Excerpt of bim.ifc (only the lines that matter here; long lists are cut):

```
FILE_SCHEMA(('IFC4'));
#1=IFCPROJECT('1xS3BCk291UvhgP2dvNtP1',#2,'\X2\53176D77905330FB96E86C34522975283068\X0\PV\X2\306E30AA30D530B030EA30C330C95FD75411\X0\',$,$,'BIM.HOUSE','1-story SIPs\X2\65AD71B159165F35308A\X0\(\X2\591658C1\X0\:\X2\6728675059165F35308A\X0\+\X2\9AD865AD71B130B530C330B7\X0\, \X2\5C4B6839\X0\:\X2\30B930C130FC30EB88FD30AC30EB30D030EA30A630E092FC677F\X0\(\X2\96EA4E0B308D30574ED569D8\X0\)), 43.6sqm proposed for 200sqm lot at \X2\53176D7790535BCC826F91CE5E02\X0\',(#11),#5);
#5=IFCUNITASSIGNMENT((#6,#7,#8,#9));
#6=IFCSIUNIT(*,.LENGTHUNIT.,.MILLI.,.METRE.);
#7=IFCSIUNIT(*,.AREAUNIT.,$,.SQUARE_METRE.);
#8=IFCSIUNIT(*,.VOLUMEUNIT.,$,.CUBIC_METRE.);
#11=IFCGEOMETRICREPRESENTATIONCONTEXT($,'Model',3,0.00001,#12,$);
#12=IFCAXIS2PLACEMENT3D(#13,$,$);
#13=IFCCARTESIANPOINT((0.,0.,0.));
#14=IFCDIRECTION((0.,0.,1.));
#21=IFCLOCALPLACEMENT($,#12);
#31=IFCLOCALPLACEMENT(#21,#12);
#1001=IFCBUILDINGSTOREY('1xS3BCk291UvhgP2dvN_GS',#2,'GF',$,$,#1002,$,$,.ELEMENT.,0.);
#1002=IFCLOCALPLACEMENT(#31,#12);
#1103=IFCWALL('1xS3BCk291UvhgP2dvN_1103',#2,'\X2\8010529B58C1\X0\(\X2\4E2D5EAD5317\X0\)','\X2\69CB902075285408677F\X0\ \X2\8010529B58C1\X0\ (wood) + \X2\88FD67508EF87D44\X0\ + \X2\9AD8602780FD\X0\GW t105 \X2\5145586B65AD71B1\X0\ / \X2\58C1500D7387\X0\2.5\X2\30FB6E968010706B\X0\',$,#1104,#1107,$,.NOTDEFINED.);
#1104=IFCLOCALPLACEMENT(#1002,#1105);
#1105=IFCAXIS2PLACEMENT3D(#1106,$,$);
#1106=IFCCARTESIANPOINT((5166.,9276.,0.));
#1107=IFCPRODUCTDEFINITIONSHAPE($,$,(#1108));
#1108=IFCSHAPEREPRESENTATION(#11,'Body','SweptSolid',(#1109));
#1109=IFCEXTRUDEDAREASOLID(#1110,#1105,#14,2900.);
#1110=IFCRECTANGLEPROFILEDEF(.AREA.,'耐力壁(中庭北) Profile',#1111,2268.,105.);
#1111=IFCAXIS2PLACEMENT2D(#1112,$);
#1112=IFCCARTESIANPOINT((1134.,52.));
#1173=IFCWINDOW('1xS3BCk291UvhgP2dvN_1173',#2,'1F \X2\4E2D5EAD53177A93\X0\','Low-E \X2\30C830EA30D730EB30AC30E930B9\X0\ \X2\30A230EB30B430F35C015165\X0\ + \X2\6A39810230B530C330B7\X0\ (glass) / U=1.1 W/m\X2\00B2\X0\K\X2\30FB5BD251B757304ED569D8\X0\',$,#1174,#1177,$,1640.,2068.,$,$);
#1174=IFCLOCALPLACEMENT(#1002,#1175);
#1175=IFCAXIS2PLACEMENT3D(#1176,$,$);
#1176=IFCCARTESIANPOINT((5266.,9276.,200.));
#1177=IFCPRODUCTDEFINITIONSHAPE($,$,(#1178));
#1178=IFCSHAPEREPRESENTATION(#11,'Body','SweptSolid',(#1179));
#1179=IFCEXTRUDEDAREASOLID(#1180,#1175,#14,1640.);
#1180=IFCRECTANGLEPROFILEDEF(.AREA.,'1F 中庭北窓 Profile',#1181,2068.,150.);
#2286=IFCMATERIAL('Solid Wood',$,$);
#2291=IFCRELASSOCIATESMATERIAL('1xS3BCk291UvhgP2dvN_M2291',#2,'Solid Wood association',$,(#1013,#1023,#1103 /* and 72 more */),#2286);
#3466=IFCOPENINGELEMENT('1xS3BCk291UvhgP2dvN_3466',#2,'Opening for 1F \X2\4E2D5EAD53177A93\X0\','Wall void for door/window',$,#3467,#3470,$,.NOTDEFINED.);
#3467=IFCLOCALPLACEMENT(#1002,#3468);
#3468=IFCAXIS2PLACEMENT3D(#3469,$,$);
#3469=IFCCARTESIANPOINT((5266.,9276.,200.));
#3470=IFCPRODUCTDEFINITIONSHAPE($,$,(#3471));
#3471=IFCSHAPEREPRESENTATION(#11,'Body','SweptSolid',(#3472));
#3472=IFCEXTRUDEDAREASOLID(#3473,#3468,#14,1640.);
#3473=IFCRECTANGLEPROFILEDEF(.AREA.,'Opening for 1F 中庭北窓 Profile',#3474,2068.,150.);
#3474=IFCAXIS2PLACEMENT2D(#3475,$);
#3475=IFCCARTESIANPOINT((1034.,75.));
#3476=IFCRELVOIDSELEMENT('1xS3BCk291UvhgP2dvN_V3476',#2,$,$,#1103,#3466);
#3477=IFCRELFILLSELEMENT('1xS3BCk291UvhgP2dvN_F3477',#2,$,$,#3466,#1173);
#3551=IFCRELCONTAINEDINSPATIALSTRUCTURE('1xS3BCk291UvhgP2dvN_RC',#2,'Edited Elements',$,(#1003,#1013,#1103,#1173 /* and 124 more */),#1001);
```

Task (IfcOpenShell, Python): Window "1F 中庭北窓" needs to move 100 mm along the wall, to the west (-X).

```python
import ifcopenshell
import ifcopenshell.api.geometry
import ifcopenshell.util.placement

model = ifcopenshell.open("bim.ifc")

window = model.by_id(1173)
opening = window.FillsVoids[0].RelatingOpeningElement
wall = opening.VoidsElements[0].RelatingBuildingElement

wall_matrix = ifcopenshell.util.placement.get_local_placement(wall.ObjectPlacement)
shift = wall_matrix[:3, 0] * -100.0
before = ifcopenshell.util.placement.get_local_placement(window.ObjectPlacement)[:3, 3].copy()

# The window is not placed relative to its opening, so move both.
for product in (opening, window):
    matrix = ifcopenshell.util.placement.get_local_placement(product.ObjectPlacement)
    matrix[:3, 3] += shift
    ifcopenshell.api.geometry.edit_object_placement(model, product=product, matrix=matrix, is_si=False)

after = ifcopenshell.util.placement.get_local_placement(window.ObjectPlacement)[:3, 3]
print("window moved by", (after - before).round(3) + 0.0)

model.write("bim_v2.ifc")
```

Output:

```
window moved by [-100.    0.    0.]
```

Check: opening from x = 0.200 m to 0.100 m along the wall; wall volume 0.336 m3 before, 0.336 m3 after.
